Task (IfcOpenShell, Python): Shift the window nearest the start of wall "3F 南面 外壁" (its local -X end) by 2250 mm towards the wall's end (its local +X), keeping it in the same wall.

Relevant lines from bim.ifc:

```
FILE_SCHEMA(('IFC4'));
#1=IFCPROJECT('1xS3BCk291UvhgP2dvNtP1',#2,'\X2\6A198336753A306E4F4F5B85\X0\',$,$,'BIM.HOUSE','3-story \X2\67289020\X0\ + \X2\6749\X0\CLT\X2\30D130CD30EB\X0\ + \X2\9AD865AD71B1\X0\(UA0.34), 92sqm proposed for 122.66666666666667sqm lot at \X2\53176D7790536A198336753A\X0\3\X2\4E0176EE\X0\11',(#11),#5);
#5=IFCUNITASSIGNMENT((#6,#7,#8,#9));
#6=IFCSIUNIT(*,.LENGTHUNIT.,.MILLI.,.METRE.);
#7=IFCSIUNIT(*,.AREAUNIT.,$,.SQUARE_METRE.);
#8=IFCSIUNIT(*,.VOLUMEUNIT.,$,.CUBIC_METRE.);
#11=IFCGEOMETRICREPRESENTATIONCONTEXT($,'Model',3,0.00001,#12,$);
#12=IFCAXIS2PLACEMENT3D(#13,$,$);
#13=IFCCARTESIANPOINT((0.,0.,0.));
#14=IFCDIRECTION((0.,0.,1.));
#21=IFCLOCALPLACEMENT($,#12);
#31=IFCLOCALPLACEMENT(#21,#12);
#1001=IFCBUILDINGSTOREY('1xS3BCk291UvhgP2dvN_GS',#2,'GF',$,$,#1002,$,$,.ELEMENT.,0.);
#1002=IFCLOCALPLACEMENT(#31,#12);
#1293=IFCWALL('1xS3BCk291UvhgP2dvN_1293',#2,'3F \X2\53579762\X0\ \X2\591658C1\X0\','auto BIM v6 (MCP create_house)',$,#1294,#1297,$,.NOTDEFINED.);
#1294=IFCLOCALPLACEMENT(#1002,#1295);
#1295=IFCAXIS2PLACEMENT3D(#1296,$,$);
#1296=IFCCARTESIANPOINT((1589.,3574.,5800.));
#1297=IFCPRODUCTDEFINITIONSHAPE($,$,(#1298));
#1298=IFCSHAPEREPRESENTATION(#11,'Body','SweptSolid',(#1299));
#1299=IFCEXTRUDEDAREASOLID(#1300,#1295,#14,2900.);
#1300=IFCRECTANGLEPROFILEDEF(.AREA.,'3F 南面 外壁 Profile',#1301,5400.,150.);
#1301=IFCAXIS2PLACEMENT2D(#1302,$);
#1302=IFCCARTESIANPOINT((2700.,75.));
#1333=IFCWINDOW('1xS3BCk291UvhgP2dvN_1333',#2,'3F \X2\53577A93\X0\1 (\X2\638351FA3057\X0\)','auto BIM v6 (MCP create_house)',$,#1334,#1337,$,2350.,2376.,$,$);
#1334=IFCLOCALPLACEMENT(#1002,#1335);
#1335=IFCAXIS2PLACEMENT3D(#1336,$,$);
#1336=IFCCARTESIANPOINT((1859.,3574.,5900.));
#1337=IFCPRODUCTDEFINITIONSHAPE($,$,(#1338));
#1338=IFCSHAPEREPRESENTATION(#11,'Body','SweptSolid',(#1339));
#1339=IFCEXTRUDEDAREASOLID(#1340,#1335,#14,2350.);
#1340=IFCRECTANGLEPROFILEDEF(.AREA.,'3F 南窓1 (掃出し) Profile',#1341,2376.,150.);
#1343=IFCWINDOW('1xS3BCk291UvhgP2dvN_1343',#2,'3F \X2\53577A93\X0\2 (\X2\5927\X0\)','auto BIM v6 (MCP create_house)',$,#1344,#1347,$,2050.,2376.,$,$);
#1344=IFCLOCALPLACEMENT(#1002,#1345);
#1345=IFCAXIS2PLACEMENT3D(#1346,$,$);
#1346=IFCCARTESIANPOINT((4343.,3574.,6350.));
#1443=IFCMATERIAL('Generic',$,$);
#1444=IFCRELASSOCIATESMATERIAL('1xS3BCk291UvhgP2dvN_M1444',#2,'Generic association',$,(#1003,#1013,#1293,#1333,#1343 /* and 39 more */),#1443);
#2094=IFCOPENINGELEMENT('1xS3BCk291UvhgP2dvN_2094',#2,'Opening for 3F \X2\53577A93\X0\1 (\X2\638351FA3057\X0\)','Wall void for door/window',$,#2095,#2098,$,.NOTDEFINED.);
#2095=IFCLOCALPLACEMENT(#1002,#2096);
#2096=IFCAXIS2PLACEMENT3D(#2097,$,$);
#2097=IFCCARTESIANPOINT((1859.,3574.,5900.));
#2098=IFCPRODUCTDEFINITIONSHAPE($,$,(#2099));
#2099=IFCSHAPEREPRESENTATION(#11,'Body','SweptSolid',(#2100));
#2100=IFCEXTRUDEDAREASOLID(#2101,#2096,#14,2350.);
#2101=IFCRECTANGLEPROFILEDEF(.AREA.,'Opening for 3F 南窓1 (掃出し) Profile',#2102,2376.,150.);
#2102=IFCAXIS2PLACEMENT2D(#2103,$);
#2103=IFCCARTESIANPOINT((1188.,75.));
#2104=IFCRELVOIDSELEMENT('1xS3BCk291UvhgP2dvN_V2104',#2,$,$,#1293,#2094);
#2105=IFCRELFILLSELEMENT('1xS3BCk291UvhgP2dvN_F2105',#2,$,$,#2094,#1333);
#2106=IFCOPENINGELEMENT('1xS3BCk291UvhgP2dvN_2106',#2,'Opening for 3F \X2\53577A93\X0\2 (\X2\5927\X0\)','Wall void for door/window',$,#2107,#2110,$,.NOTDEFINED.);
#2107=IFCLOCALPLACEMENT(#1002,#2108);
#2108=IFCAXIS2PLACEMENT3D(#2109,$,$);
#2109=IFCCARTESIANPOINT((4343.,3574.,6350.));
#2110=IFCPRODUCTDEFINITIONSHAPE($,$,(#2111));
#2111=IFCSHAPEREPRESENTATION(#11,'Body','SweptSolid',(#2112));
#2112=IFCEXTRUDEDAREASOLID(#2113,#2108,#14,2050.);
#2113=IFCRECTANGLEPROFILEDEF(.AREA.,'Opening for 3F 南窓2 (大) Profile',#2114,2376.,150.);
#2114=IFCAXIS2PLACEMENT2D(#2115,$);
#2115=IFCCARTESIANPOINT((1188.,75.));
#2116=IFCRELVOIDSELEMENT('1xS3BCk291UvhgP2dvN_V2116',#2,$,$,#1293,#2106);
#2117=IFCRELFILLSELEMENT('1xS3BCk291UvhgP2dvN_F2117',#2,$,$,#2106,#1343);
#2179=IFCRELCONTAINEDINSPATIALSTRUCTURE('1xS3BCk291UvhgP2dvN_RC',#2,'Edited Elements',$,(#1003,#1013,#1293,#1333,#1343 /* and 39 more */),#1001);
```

```python
import ifcopenshell
import ifcopenshell.api.geometry
import ifcopenshell.util.placement

model = ifcopenshell.open("bim.ifc")

window = model.by_guid("1xS3BCk291UvhgP2dvN_1333")
opening = window.FillsVoids[0].RelatingOpeningElement
wall = opening.VoidsElements[0].RelatingBuildingElement

wall_matrix = ifcopenshell.util.placement.get_local_placement(wall.ObjectPlacement)
shift = wall_matrix[:3, 0] * 2250.0
before = ifcopenshell.util.placement.get_local_placement(window.ObjectPlacement)[:3, 3].copy()

# The window is not placed relative to its opening, so move both.
for product in (opening, window):
    matrix = ifcopenshell.util.placement.get_local_placement(product.ObjectPlacement)
    matrix[:3, 3] += shift
    ifcopenshell.api.geometry.edit_object_placement(model, product=product, matrix=matrix, is_si=False)

after = ifcopenshell.util.placement.get_local_placement(window.ObjectPlacement)[:3, 3]
print("window moved by", (after - before).round(3) + 0.0)

model.write("bim_updated.ifc")
```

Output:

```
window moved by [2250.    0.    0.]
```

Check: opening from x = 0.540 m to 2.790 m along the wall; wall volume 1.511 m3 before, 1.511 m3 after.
